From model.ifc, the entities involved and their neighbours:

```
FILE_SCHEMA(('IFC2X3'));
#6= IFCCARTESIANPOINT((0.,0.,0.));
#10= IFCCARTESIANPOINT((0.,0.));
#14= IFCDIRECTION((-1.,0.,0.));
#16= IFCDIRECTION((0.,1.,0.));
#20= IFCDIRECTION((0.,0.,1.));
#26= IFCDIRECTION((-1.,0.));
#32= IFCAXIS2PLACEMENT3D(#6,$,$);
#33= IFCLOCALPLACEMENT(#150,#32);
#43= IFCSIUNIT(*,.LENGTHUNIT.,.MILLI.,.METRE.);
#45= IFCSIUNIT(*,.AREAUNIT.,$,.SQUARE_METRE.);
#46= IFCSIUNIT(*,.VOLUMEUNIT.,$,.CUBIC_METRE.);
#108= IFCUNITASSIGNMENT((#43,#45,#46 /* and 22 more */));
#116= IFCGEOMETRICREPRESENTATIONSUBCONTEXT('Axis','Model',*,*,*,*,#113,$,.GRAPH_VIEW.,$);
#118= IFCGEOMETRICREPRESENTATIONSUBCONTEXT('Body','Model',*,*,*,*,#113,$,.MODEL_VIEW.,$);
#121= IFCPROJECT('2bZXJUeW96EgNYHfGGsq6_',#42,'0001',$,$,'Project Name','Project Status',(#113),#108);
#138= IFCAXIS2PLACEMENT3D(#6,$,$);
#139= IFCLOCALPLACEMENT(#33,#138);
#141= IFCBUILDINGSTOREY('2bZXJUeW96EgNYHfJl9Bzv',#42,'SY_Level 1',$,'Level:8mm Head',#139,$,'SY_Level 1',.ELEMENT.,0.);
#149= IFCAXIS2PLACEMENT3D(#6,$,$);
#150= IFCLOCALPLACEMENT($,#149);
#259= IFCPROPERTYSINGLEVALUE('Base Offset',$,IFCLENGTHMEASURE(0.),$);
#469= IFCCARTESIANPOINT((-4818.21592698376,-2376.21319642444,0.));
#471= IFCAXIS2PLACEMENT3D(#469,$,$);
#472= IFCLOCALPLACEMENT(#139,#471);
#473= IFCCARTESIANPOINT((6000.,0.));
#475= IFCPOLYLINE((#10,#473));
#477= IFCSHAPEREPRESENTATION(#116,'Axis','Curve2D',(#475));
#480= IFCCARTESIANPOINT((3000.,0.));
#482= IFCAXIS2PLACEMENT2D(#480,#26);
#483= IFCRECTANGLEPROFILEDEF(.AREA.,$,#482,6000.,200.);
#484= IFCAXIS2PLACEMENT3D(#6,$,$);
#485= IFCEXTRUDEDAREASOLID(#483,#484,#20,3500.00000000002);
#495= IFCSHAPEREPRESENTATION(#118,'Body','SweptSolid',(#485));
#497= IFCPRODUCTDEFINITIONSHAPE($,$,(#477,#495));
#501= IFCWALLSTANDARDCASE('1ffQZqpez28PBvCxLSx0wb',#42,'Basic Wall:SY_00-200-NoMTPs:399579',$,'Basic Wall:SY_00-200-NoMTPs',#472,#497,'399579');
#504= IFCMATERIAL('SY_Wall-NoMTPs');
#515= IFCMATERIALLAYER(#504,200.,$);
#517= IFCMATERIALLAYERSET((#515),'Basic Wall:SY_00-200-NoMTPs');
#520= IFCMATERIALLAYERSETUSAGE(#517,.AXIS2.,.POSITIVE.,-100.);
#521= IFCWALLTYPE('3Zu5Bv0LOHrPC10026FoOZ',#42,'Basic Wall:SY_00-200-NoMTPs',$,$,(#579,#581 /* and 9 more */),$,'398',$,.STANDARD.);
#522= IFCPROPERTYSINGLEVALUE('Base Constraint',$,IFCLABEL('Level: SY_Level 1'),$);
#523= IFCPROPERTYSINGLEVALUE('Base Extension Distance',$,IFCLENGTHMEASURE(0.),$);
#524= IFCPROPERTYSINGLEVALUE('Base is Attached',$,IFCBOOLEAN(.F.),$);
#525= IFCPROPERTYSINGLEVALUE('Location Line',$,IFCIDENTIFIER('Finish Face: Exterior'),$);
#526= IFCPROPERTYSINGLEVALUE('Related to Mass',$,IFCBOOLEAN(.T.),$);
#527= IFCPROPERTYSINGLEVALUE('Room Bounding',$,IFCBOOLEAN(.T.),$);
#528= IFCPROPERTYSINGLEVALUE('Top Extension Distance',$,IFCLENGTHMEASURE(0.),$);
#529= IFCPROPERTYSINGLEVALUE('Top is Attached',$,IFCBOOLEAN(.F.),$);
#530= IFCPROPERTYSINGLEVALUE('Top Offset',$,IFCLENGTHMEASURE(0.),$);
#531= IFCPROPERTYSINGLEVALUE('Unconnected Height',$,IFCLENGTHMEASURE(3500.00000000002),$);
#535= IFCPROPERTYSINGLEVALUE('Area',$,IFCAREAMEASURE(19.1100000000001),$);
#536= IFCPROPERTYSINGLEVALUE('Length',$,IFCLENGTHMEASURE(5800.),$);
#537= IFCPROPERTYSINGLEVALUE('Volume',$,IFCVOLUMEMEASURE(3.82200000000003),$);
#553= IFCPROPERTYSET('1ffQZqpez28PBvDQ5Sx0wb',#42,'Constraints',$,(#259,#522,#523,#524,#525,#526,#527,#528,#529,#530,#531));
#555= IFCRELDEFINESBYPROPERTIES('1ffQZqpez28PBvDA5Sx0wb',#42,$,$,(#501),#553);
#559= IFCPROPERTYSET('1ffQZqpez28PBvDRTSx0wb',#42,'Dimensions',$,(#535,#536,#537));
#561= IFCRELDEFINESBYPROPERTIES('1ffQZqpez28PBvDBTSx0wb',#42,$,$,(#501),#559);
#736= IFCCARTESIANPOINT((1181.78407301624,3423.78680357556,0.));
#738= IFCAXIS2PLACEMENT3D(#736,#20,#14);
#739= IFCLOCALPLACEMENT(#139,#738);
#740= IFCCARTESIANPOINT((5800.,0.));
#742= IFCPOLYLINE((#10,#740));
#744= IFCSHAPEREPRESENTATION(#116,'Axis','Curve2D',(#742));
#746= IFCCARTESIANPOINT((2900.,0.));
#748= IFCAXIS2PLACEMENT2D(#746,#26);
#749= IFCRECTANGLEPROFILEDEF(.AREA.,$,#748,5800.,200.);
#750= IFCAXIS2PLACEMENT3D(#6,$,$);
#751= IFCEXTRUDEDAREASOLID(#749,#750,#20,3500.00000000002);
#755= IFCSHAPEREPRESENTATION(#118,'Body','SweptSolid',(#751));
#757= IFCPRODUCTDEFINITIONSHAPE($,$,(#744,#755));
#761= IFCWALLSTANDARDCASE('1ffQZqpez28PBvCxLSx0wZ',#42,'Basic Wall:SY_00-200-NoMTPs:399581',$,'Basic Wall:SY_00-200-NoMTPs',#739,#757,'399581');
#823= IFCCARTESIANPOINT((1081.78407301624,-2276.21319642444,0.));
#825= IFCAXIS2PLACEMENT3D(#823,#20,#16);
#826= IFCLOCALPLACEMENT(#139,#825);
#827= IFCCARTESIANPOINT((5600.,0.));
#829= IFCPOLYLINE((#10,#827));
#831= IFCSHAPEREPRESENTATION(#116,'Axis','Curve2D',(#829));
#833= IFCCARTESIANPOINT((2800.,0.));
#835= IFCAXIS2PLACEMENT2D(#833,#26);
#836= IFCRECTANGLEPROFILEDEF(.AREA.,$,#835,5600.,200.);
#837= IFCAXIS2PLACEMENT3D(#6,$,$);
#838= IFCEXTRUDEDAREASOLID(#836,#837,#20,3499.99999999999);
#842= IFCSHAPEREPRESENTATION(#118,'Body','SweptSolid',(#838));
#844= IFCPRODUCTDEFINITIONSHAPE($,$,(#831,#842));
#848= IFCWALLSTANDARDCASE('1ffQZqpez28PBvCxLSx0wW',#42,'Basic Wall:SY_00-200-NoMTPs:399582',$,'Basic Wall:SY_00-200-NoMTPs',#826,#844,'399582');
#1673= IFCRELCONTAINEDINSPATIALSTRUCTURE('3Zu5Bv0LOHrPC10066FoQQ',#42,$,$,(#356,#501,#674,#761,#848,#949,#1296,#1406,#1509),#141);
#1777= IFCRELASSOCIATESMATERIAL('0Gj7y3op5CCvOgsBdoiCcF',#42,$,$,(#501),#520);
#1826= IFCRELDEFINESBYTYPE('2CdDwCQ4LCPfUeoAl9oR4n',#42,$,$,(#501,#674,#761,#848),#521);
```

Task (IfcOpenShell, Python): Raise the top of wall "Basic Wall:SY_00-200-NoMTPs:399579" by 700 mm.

```python
import ifcopenshell
import ifcopenshell.api.pset
import ifcopenshell.geom
import ifcopenshell.util.element
import ifcopenshell.util.representation
import ifcopenshell.util.shape
import ifcopenshell.util.unit

model = ifcopenshell.open("model.ifc")
unit_scale = ifcopenshell.util.unit.calculate_unit_scale(model)
area_scale = ifcopenshell.util.unit.calculate_unit_scale(model, "AREAUNIT")
volume_scale = ifcopenshell.util.unit.calculate_unit_scale(model, "VOLUMEUNIT")
settings = ifcopenshell.geom.settings()


def volume(element):
    """Net volume in cubic metres, openings subtracted."""
    shape = ifcopenshell.geom.create_shape(settings, element)
    return ifcopenshell.util.shape.get_volume(shape.geometry)


wall = model.by_id(501)
before = volume(wall)

body = ifcopenshell.util.representation.get_representation(wall, "Model", "Body")
solid = body.Items[0]
old_height = solid.Depth
solid.Depth += 0.7 / unit_scale
after = volume(wall)
thickness = 0.2  # wall thickness in metres

# Update the stored height, areas and volumes.
pset = model.by_id(ifcopenshell.util.element.get_pset(wall, "Constraints", should_inherit=False)["id"])
ifcopenshell.api.pset.edit_pset(model, pset=pset, properties={
    "Unconnected Height": model.create_entity("IfcLengthMeasure", solid.Depth),
})
pset = model.by_id(ifcopenshell.util.element.get_pset(wall, "Dimensions", should_inherit=False)["id"])
ifcopenshell.api.pset.edit_pset(model, pset=pset, properties={
    "Area": model.create_entity("IfcAreaMeasure", after / thickness / area_scale),
    "Volume": model.create_entity("IfcVolumeMeasure", after / volume_scale),
})

print(f"height {old_height:g} -> {solid.Depth:g}, volume {before:.3f} -> {after:.3f} m3")

model.write("model_rev.ifc")
```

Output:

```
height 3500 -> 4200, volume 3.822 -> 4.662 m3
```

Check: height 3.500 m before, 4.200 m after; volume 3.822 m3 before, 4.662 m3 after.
